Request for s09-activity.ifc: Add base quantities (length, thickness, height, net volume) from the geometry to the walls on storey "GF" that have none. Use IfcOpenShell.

First a look at what the model holds.

```python
import ifcopenshell
import ifcopenshell.util.element
import ifcopenshell.util.unit

model = ifcopenshell.open("s09-activity.ifc")
print(model.schema)
for unit_type in ("LENGTHUNIT", "AREAUNIT", "VOLUMEUNIT"):
    print(unit_type, ifcopenshell.util.unit.calculate_unit_scale(model, unit_type))
storey = next(s for s in model.by_type("IfcBuildingStorey") if s.Name == "GF")
walls = [e for e in ifcopenshell.util.element.get_decomposition(storey) if e.is_a("IfcWall")]
for e in sorted(walls, key=lambda e: e.id()):
    print(e.id(), e.is_a(), e.Name, list(ifcopenshell.util.element.get_psets(e, qtos_only=True)), sep=" | ")
```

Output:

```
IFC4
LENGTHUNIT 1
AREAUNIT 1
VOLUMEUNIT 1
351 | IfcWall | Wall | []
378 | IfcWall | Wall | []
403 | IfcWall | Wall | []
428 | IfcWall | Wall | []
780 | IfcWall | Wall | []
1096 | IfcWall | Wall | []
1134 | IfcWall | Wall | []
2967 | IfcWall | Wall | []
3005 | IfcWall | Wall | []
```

```python
import ifcopenshell
import ifcopenshell.api.pset
import ifcopenshell.geom
import ifcopenshell.util.element
import ifcopenshell.util.shape
import ifcopenshell.util.unit

model = ifcopenshell.open("s09-activity.ifc")
unit_scale = ifcopenshell.util.unit.calculate_unit_scale(model)
volume_scale = ifcopenshell.util.unit.calculate_unit_scale(model, "VOLUMEUNIT")
settings = ifcopenshell.geom.settings()

storey = next(s for s in model.by_type("IfcBuildingStorey") if s.Name == "GF")
walls = [e for e in ifcopenshell.util.element.get_decomposition(storey) if e.is_a("IfcWall")]

for e in sorted(walls, key=lambda e: e.id()):
    if ifcopenshell.util.element.get_psets(e, qtos_only=True, should_inherit=False):
        continue
    # Geometry comes back in metres, in the element's own axes.
    shape = ifcopenshell.geom.create_shape(settings, e)
    values = {
        "Length": ifcopenshell.util.shape.get_x(shape.geometry) / unit_scale,
        "Width": ifcopenshell.util.shape.get_y(shape.geometry) / unit_scale,
        "Height": ifcopenshell.util.shape.get_z(shape.geometry) / unit_scale,
        "NetVolume": ifcopenshell.util.shape.get_volume(shape.geometry) / volume_scale,
    }
    qto = ifcopenshell.api.pset.add_qto(model, product=e, name="Qto_WallBaseQuantities")
    ifcopenshell.api.pset.edit_qto(model, qto=qto, properties=values)
    print(e.id(), {k: round(v, 3) for k, v in values.items()})

model.write("s09-activity_updated.ifc")
```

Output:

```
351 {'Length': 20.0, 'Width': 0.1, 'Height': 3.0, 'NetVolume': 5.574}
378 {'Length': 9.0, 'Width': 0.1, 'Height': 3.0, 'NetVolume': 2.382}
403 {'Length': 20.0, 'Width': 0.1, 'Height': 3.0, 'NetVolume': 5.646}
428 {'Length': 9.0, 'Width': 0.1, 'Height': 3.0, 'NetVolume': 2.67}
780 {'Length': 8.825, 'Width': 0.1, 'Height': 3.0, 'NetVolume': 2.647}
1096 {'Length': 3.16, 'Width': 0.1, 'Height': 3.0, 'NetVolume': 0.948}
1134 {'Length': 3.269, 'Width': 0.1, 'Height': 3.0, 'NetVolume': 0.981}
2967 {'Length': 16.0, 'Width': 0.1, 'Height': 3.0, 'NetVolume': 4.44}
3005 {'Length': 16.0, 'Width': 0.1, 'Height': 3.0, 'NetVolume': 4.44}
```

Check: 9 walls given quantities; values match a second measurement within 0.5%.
